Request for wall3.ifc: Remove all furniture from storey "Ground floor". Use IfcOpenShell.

First a look at what the model holds.

```python
import ifcopenshell
import ifcopenshell.util.element

model = ifcopenshell.open("wall3.ifc")
print(model.schema)
storey = next(s for s in model.by_type("IfcBuildingStorey") if s.Name == "Ground floor")
furniture = [e for e in ifcopenshell.util.element.get_decomposition(storey) if e.is_a("IfcFurnishingElement")]
seen = {}
for e in furniture:
    element_type = ifcopenshell.util.element.get_type(e)
    name = element_type.Name if element_type not in (None, e) else None
    seen[name] = seen.get(name, 0) + 1
for name, count in sorted(seen.items(), key=str):
    print(count, "x", name)
```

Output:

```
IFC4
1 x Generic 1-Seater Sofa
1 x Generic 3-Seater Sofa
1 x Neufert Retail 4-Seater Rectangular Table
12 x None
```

```python
import ifcopenshell
import ifcopenshell.api.root
import ifcopenshell.util.element

model = ifcopenshell.open("wall3.ifc")

storey = next(s for s in model.by_type("IfcBuildingStorey") if s.Name == "Ground floor")
furniture = [e for e in ifcopenshell.util.element.get_decomposition(storey) if e.is_a("IfcFurnishingElement")]

for e in furniture:
    ifcopenshell.api.root.remove_product(model, product=e)
print(len(furniture), "removed")

model.write("wall3_updated.ifc")
```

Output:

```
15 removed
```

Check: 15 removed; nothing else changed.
